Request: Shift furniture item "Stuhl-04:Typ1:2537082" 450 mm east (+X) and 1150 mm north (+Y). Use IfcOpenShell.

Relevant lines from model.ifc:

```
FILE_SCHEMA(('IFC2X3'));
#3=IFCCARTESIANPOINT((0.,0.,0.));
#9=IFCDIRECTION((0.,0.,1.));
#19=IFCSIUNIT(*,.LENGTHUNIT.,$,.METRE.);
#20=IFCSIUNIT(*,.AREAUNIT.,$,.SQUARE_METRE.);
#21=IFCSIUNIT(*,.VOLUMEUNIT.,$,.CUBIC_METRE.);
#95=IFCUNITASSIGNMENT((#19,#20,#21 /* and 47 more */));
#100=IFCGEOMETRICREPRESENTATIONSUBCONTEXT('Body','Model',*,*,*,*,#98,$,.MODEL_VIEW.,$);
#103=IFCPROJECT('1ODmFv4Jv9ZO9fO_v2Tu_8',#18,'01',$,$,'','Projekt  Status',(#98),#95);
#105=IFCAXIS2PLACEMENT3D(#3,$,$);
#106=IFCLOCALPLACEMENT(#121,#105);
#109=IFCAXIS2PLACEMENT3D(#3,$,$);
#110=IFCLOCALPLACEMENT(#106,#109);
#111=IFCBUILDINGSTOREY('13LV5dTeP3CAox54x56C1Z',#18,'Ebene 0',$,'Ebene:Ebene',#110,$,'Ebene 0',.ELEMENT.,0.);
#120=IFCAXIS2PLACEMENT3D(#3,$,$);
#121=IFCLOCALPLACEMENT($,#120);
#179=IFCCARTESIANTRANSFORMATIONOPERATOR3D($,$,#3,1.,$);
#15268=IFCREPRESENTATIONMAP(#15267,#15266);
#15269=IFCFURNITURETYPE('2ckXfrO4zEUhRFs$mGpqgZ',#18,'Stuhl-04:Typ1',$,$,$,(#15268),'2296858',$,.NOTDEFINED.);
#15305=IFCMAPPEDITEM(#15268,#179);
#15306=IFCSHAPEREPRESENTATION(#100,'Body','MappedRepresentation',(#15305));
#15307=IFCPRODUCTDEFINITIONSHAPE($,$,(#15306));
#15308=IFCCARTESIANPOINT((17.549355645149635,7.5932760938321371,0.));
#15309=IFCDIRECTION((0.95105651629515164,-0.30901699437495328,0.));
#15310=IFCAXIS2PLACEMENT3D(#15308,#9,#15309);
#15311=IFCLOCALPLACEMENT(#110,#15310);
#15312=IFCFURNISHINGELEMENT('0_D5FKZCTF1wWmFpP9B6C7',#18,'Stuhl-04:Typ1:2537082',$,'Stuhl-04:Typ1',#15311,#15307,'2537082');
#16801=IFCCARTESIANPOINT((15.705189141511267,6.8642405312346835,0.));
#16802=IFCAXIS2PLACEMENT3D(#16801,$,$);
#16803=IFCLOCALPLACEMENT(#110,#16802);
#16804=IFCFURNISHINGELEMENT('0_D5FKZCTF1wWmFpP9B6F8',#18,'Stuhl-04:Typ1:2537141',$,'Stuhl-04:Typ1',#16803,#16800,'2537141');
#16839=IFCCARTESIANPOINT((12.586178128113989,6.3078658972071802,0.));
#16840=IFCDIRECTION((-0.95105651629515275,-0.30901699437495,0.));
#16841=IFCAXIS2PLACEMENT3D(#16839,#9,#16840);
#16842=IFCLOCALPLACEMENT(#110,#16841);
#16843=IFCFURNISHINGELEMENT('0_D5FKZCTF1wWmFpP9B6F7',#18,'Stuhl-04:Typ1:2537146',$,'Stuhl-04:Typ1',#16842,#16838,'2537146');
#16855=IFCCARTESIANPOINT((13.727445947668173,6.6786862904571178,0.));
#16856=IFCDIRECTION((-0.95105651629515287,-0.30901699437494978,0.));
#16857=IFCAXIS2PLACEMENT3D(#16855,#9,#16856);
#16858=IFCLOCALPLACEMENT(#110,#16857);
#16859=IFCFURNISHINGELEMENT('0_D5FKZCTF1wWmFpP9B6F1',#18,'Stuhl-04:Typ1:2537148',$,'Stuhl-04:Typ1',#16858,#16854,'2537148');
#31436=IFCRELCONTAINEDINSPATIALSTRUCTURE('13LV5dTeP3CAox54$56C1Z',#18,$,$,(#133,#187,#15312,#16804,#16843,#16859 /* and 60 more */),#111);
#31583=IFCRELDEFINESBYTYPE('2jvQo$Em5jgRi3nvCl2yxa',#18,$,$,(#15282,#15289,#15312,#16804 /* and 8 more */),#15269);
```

```python
import ifcopenshell
import ifcopenshell.api.geometry
import ifcopenshell.util.placement
import ifcopenshell.util.unit

model = ifcopenshell.open("model.ifc")
unit_scale = ifcopenshell.util.unit.calculate_unit_scale(model)

item = model.by_guid("0_D5FKZCTF1wWmFpP9B6C7")
matrix = ifcopenshell.util.placement.get_local_placement(item.ObjectPlacement)
matrix[0, 3] += 0.45 / unit_scale
matrix[1, 3] += 1.15 / unit_scale
ifcopenshell.api.geometry.edit_object_placement(model, product=item, matrix=matrix, is_si=False)

print(ifcopenshell.util.placement.get_local_placement(item.ObjectPlacement).round(3) + 0.0)

model.write("model_edited.ifc")
```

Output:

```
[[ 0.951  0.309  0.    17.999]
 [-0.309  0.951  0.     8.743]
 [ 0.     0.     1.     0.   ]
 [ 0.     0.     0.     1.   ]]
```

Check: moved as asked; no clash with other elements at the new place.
